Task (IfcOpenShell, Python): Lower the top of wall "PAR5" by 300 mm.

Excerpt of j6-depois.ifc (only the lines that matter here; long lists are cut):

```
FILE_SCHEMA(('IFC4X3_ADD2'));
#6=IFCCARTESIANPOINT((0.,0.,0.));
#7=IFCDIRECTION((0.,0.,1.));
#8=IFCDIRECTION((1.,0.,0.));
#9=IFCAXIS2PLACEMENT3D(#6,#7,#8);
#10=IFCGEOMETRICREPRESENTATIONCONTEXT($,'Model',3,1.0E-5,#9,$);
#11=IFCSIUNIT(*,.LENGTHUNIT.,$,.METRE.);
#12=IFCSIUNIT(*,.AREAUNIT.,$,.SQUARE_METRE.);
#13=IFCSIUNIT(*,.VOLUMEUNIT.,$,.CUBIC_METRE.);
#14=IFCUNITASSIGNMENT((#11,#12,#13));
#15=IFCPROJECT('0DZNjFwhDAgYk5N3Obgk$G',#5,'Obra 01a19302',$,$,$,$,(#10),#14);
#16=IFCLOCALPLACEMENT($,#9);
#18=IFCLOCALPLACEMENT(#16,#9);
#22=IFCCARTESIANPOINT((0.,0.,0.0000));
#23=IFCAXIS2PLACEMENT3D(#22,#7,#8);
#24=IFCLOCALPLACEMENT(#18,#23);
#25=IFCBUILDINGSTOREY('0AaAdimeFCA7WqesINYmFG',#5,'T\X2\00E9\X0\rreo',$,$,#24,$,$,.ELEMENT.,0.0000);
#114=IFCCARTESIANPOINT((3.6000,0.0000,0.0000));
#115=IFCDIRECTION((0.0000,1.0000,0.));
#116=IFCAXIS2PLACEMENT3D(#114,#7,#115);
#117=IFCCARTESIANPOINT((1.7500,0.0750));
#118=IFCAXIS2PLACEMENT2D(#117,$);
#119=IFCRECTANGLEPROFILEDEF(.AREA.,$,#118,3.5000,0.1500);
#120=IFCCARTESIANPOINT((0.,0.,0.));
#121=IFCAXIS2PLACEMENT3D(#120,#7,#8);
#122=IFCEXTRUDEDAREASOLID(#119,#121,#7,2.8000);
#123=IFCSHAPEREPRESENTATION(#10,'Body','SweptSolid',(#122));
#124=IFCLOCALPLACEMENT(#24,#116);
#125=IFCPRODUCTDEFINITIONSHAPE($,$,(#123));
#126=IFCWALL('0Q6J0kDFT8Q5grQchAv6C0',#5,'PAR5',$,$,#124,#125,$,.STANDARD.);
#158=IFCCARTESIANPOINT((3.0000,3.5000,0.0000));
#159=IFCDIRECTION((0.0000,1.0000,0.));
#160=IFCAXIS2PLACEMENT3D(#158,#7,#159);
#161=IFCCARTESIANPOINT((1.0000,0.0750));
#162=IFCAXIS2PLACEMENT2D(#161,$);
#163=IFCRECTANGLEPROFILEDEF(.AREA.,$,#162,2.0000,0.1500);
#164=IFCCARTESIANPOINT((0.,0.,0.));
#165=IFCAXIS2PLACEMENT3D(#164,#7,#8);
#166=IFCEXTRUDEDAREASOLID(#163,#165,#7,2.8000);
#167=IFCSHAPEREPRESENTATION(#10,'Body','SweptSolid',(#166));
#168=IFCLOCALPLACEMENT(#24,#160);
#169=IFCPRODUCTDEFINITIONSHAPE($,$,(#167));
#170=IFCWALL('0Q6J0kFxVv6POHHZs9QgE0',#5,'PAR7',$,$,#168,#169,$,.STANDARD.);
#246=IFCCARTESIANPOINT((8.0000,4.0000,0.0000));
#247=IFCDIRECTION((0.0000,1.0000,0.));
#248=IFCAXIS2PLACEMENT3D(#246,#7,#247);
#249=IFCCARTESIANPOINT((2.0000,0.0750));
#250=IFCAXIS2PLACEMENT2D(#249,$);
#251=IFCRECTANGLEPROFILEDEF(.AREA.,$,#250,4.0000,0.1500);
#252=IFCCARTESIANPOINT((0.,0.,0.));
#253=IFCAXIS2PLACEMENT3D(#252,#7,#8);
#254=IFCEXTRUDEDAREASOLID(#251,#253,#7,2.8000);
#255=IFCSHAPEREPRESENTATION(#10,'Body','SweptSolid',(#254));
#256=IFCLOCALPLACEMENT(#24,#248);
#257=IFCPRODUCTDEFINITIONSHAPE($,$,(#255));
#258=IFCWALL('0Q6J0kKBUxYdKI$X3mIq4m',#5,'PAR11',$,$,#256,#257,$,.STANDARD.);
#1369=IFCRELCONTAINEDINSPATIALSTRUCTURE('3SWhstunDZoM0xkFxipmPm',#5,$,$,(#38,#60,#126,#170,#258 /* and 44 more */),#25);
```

```python
import ifcopenshell
import ifcopenshell.geom
import ifcopenshell.util.shape

model = ifcopenshell.open("j6-depois.ifc")
settings = ifcopenshell.geom.settings()


def volume(element):
    """Net volume in cubic metres, openings subtracted."""
    shape = ifcopenshell.geom.create_shape(settings, element)
    return ifcopenshell.util.shape.get_volume(shape.geometry)


wall = model.by_id(126)
before = volume(wall)

body = next(r for r in wall.Representation.Representations if r.RepresentationIdentifier == "Body")
solid = body.Items[0]
old_height = solid.Depth
solid.Depth -= 0.3
after = volume(wall)

print(f"height {old_height:g} -> {solid.Depth:g}, volume {before:.3f} -> {after:.3f} m3")

model.write("j6-depois_v2.ifc")
```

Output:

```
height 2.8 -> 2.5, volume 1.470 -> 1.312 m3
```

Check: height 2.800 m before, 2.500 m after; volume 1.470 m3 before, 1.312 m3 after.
